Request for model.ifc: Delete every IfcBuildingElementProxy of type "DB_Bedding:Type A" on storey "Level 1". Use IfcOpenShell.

First a look at what the model holds.

```python
import ifcopenshell
import ifcopenshell.util.element

model = ifcopenshell.open("model.ifc")
print(model.schema)
storey = next(s for s in model.by_type("IfcBuildingStorey") if s.Name == "Level 1")
proxies = [e for e in ifcopenshell.util.element.get_decomposition(storey) if e.is_a("IfcBuildingElementProxy")]
seen = {}
for e in proxies:
    element_type = ifcopenshell.util.element.get_type(e)
    name = element_type.Name if element_type not in (None, e) else None
    seen[name] = seen.get(name, 0) + 1
for name, count in sorted(seen.items(), key=str):
    print(count, "x", name)
```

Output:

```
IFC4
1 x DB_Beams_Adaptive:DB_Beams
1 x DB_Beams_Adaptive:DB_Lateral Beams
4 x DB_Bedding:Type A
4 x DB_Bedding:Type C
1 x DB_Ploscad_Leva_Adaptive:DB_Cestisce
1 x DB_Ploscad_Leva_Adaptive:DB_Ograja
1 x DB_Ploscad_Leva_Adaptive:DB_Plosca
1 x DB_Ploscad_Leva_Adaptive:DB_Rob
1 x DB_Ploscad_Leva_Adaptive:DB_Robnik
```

```python
import ifcopenshell
import ifcopenshell.api.root
import ifcopenshell.util.element

model = ifcopenshell.open("model.ifc")

storey = next(s for s in model.by_type("IfcBuildingStorey") if s.Name == "Level 1")
proxies = [e for e in ifcopenshell.util.element.get_decomposition(storey) if e.is_a("IfcBuildingElementProxy")]
targets = [e for e in proxies if (t := ifcopenshell.util.element.get_type(e)) not in (None, e) and t.Name == "DB_Bedding:Type A"]

for e in targets:
    ifcopenshell.api.root.remove_product(model, product=e)
print(len(targets), "removed")

model.write("model_rev.ifc")
```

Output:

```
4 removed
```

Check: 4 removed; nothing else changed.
